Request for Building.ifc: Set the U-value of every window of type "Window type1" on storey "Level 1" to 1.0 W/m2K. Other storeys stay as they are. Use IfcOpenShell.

First a look at what the model holds.

```python
import ifcopenshell
import ifcopenshell.util.element

model = ifcopenshell.open("Building.ifc")
print(model.schema)
storey = next(s for s in model.by_type("IfcBuildingStorey") if s.Name == "Level 1")
windows = [e for e in ifcopenshell.util.element.get_decomposition(storey) if e.is_a("IfcWindow")]
seen = {}
for e in windows:
    element_type = ifcopenshell.util.element.get_type(e)
    key = (element_type.Name if element_type != e and element_type else None, ifcopenshell.util.element.get_pset(e, "Pset_WindowCommon", "ThermalTransmittance"))
    seen[key] = seen.get(key, 0) + 1
for (name, value), count in sorted(seen.items(), key=str):
    print(count, "x", name, "|", value)
```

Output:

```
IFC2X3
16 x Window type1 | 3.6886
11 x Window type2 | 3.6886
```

```python
import ifcopenshell
import ifcopenshell.api.pset
import ifcopenshell.util.element

model = ifcopenshell.open("Building.ifc")

storey = next(s for s in model.by_type("IfcBuildingStorey") if s.Name == "Level 1")
windows = [e for e in ifcopenshell.util.element.get_decomposition(storey) if e.is_a("IfcWindow")]

count = 0
for e in windows:
    element_type = ifcopenshell.util.element.get_type(e)
    if element_type in (None, e) or element_type.Name != "Window type1":
        continue
    # add_pset returns the element's existing set when there is one.
    pset = ifcopenshell.api.pset.add_pset(model, product=e, name="Pset_WindowCommon")
    ifcopenshell.api.pset.edit_pset(model, pset=pset, properties={"ThermalTransmittance": 1.0})
    count += 1

print(count, "windows updated")

model.write("Building_edited.ifc")
```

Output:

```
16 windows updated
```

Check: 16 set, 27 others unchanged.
